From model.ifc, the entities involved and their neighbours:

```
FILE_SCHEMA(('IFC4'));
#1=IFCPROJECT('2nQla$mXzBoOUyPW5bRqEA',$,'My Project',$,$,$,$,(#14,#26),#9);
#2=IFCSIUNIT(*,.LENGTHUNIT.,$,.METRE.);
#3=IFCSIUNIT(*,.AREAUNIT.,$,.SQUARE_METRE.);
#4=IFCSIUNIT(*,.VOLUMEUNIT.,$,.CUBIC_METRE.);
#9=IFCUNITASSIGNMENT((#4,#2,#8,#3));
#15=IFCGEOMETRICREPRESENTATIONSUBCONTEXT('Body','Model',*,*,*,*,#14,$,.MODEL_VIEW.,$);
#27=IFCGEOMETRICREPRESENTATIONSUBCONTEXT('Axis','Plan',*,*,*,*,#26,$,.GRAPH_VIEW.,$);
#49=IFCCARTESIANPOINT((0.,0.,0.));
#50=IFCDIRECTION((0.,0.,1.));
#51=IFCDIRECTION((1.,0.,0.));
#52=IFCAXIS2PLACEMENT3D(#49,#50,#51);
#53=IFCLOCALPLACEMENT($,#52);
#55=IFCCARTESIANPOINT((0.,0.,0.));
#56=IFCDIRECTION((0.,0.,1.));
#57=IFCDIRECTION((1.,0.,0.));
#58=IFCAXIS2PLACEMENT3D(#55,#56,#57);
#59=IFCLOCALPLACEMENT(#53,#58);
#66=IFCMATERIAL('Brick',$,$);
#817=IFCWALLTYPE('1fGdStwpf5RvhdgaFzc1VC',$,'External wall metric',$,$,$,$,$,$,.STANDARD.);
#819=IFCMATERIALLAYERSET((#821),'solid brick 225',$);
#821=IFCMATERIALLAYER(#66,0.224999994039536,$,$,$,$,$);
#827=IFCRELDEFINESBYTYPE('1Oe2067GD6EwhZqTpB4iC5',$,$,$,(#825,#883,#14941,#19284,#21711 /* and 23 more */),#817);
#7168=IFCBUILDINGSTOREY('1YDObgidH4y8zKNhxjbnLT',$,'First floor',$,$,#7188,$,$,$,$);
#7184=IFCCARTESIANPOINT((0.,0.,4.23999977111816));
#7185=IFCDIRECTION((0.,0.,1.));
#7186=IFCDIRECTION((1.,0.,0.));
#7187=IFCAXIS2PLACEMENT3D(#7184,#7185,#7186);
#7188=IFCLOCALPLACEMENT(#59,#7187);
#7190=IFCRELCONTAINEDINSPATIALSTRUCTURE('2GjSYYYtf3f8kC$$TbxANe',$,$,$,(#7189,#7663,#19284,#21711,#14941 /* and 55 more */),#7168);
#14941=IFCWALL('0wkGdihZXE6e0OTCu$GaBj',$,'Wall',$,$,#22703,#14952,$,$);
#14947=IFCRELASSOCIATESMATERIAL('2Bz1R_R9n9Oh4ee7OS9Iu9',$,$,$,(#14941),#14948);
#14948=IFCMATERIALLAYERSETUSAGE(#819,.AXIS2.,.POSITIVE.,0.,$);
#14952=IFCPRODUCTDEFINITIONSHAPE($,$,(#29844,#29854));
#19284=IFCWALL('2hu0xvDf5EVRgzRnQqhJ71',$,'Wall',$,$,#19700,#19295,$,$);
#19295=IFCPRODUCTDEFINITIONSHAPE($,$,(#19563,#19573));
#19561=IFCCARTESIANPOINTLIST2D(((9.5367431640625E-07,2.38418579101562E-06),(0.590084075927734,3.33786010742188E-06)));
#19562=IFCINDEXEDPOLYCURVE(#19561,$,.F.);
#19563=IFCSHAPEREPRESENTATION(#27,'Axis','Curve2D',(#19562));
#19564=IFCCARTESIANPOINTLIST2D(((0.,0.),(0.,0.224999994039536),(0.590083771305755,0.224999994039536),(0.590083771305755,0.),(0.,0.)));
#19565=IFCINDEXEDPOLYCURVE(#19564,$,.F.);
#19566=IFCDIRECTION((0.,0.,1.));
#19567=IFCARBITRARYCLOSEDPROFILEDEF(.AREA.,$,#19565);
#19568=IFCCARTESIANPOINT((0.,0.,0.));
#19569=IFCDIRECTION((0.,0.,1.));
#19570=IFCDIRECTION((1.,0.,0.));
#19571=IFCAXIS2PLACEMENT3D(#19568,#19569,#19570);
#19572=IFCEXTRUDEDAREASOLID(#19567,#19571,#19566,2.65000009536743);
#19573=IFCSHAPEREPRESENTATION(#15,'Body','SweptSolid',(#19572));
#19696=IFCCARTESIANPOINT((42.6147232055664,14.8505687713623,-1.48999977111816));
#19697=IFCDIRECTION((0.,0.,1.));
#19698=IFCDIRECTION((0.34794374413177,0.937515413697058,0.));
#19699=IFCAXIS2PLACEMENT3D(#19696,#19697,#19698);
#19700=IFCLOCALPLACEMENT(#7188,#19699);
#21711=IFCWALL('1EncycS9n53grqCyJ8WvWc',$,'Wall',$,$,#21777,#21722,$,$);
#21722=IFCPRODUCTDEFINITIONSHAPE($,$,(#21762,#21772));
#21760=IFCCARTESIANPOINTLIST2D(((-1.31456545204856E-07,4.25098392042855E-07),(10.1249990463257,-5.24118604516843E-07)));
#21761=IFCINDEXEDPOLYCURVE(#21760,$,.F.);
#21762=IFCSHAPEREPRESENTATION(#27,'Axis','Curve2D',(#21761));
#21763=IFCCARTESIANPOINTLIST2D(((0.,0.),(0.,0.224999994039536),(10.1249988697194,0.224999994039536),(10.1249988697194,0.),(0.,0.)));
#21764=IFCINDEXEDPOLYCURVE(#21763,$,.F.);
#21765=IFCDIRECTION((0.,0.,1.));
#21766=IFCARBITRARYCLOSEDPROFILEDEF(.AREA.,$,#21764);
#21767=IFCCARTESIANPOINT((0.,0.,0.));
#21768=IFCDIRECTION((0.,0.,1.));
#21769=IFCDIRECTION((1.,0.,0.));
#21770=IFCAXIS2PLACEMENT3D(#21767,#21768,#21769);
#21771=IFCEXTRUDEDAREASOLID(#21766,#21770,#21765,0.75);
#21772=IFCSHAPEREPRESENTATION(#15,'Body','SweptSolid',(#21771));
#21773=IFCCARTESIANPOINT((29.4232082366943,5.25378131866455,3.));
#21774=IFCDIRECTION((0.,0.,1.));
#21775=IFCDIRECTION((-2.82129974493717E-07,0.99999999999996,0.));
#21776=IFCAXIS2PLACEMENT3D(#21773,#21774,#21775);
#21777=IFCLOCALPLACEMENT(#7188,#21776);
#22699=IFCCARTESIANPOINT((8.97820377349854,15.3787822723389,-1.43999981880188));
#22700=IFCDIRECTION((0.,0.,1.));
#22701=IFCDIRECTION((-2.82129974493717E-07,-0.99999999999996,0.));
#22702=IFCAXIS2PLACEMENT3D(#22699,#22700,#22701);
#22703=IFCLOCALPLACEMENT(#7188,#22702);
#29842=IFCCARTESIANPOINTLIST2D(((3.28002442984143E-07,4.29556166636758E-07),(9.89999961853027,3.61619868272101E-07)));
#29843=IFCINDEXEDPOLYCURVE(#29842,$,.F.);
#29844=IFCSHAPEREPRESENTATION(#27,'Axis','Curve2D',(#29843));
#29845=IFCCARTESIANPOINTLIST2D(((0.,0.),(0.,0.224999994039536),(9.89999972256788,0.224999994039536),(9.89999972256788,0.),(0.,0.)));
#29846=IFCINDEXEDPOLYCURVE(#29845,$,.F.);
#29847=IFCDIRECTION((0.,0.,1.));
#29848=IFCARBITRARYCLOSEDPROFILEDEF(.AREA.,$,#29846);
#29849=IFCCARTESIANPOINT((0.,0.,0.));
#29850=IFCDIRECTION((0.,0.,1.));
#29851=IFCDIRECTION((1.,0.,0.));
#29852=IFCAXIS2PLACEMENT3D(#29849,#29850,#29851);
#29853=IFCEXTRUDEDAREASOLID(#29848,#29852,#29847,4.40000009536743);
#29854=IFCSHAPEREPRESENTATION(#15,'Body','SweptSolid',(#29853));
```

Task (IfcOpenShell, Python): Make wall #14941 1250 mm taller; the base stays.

```python
import ifcopenshell
import ifcopenshell.geom
import ifcopenshell.util.representation
import ifcopenshell.util.shape
import ifcopenshell.util.unit

model = ifcopenshell.open("model.ifc")
unit_scale = ifcopenshell.util.unit.calculate_unit_scale(model)
settings = ifcopenshell.geom.settings()


def volume(element):
    """Net volume in cubic metres, openings subtracted."""
    shape = ifcopenshell.geom.create_shape(settings, element)
    return ifcopenshell.util.shape.get_volume(shape.geometry)


wall = model.by_guid("0wkGdihZXE6e0OTCu$GaBj")
before = volume(wall)

body = ifcopenshell.util.representation.get_representation(wall, "Model", "Body")
solid = body.Items[0]
old_height = solid.Depth
solid.Depth += 1.25 / unit_scale
after = volume(wall)

print(f"height {old_height:g} -> {solid.Depth:g}, volume {before:.3f} -> {after:.3f} m3")

model.write("model-out.ifc")
```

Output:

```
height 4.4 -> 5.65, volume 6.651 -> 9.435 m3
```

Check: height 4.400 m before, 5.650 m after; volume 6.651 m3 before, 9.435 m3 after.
